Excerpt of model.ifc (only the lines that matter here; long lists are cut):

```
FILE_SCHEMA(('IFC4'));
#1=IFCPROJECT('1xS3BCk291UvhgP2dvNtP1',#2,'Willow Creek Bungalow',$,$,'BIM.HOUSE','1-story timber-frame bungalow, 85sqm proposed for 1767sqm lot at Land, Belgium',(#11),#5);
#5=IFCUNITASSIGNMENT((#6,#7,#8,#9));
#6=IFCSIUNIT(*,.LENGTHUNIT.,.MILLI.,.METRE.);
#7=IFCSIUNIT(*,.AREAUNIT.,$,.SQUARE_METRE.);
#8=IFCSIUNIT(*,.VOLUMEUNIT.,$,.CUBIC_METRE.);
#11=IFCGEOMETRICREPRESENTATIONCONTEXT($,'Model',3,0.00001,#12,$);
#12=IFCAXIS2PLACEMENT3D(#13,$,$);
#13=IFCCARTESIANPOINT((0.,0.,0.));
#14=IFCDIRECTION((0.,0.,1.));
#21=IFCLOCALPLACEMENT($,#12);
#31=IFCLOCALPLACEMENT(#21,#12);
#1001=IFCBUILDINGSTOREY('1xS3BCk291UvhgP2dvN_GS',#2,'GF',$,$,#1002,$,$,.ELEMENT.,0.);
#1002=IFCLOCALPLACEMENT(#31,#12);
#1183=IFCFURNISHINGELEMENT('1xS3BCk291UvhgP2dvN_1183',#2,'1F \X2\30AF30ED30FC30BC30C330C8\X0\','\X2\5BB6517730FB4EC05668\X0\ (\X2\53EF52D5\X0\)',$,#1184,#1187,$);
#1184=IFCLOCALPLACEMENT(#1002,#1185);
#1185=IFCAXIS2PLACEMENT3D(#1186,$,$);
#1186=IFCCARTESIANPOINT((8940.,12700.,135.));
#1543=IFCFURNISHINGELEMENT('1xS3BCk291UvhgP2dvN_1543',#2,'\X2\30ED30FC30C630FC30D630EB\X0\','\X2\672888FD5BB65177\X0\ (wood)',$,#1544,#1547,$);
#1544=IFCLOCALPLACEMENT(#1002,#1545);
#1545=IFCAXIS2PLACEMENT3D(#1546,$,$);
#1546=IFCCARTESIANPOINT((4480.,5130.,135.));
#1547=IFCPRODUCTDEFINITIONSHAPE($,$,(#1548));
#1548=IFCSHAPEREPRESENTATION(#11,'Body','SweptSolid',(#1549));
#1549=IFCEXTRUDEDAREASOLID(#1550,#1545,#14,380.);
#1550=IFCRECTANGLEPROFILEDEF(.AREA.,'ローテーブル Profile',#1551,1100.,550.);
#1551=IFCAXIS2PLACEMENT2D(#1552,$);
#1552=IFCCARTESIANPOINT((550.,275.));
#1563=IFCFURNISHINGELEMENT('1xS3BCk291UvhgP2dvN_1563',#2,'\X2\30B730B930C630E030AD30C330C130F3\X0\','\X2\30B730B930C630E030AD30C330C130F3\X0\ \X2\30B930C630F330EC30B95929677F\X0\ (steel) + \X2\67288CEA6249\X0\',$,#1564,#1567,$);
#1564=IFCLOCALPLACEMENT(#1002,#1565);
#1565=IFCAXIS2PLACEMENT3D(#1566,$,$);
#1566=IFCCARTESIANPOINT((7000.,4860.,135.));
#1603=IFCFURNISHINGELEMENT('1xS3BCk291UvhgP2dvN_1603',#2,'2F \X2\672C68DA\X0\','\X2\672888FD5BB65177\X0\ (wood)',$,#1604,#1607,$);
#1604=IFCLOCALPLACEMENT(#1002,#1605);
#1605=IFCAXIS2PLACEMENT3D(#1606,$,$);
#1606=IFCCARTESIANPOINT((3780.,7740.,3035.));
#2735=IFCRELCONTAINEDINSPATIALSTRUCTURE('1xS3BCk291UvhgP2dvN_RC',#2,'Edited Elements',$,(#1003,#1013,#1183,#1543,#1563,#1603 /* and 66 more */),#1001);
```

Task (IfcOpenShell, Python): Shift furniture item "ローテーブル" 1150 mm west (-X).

```python
import ifcopenshell
import ifcopenshell.api.geometry
import ifcopenshell.util.placement
import ifcopenshell.util.unit

model = ifcopenshell.open("model.ifc")
unit_scale = ifcopenshell.util.unit.calculate_unit_scale(model)

item = model.by_guid("1xS3BCk291UvhgP2dvN_1543")
matrix = ifcopenshell.util.placement.get_local_placement(item.ObjectPlacement)
matrix[0, 3] -= 1.15 / unit_scale
ifcopenshell.api.geometry.edit_object_placement(model, product=item, matrix=matrix, is_si=False)

print(ifcopenshell.util.placement.get_local_placement(item.ObjectPlacement).round(3) + 0.0)

model.write("model_v2.ifc")
```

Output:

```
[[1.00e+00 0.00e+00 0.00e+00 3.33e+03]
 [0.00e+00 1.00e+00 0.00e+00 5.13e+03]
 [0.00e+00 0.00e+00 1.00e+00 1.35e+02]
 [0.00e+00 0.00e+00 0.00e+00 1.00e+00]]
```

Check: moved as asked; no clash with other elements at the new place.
